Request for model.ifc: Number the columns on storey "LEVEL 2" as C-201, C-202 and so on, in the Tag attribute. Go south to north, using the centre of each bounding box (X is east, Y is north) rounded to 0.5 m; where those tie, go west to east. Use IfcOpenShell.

First a look at what the model holds.

```python
import ifcopenshell
import ifcopenshell.util.element
import ifcopenshell.util.placement

model = ifcopenshell.open("model.ifc")
print(model.schema)
storey = next(s for s in model.by_type("IfcBuildingStorey") if s.Name == "LEVEL 2")
columns = [e for e in ifcopenshell.util.element.get_decomposition(storey) if e.is_a("IfcColumn")]
for e in sorted(columns, key=lambda e: e.id()):
    origin = ifcopenshell.util.placement.get_local_placement(e.ObjectPlacement)[:3, 3]
    print(e.id(), e.Tag, e.Name, origin.round(2) + 0.0, sep=" | ")
```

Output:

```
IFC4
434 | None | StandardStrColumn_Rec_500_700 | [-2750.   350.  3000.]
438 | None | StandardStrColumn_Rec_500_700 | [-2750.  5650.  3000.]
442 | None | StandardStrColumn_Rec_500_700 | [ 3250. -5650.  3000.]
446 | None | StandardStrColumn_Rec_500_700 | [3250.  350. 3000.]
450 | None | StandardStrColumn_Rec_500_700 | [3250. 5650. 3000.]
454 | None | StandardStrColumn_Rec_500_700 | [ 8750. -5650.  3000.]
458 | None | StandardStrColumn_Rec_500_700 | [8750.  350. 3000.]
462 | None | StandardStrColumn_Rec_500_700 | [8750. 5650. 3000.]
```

```python
import ifcopenshell
import ifcopenshell.geom
import ifcopenshell.util.element
import ifcopenshell.util.shape

model = ifcopenshell.open("model.ifc")
settings = ifcopenshell.geom.settings()
settings.set("use-world-coords", True)


def centre(element):
    shape = ifcopenshell.geom.create_shape(settings, element)
    return ifcopenshell.util.shape.get_bbox_centroid(shape.geometry)


storey = next(s for s in model.by_type("IfcBuildingStorey") if s.Name == "LEVEL 2")
columns = [e for e in ifcopenshell.util.element.get_decomposition(storey) if e.is_a("IfcColumn")]

# Insertion points can sit at a corner or the storey origin, so sort by the geometry (in metres).
centres = {e: centre(e) for e in columns}
columns.sort(key=lambda e: (round(centres[e][1] / 0.5), centres[e][0]))

for i, e in enumerate(columns, start=1):
    number = f"C-2{i:02d}"
    e.Tag = number
    print(e.id(), number)

model.write("model-out.ifc")
```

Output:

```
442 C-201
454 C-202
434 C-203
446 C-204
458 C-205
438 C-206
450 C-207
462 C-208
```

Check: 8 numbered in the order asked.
